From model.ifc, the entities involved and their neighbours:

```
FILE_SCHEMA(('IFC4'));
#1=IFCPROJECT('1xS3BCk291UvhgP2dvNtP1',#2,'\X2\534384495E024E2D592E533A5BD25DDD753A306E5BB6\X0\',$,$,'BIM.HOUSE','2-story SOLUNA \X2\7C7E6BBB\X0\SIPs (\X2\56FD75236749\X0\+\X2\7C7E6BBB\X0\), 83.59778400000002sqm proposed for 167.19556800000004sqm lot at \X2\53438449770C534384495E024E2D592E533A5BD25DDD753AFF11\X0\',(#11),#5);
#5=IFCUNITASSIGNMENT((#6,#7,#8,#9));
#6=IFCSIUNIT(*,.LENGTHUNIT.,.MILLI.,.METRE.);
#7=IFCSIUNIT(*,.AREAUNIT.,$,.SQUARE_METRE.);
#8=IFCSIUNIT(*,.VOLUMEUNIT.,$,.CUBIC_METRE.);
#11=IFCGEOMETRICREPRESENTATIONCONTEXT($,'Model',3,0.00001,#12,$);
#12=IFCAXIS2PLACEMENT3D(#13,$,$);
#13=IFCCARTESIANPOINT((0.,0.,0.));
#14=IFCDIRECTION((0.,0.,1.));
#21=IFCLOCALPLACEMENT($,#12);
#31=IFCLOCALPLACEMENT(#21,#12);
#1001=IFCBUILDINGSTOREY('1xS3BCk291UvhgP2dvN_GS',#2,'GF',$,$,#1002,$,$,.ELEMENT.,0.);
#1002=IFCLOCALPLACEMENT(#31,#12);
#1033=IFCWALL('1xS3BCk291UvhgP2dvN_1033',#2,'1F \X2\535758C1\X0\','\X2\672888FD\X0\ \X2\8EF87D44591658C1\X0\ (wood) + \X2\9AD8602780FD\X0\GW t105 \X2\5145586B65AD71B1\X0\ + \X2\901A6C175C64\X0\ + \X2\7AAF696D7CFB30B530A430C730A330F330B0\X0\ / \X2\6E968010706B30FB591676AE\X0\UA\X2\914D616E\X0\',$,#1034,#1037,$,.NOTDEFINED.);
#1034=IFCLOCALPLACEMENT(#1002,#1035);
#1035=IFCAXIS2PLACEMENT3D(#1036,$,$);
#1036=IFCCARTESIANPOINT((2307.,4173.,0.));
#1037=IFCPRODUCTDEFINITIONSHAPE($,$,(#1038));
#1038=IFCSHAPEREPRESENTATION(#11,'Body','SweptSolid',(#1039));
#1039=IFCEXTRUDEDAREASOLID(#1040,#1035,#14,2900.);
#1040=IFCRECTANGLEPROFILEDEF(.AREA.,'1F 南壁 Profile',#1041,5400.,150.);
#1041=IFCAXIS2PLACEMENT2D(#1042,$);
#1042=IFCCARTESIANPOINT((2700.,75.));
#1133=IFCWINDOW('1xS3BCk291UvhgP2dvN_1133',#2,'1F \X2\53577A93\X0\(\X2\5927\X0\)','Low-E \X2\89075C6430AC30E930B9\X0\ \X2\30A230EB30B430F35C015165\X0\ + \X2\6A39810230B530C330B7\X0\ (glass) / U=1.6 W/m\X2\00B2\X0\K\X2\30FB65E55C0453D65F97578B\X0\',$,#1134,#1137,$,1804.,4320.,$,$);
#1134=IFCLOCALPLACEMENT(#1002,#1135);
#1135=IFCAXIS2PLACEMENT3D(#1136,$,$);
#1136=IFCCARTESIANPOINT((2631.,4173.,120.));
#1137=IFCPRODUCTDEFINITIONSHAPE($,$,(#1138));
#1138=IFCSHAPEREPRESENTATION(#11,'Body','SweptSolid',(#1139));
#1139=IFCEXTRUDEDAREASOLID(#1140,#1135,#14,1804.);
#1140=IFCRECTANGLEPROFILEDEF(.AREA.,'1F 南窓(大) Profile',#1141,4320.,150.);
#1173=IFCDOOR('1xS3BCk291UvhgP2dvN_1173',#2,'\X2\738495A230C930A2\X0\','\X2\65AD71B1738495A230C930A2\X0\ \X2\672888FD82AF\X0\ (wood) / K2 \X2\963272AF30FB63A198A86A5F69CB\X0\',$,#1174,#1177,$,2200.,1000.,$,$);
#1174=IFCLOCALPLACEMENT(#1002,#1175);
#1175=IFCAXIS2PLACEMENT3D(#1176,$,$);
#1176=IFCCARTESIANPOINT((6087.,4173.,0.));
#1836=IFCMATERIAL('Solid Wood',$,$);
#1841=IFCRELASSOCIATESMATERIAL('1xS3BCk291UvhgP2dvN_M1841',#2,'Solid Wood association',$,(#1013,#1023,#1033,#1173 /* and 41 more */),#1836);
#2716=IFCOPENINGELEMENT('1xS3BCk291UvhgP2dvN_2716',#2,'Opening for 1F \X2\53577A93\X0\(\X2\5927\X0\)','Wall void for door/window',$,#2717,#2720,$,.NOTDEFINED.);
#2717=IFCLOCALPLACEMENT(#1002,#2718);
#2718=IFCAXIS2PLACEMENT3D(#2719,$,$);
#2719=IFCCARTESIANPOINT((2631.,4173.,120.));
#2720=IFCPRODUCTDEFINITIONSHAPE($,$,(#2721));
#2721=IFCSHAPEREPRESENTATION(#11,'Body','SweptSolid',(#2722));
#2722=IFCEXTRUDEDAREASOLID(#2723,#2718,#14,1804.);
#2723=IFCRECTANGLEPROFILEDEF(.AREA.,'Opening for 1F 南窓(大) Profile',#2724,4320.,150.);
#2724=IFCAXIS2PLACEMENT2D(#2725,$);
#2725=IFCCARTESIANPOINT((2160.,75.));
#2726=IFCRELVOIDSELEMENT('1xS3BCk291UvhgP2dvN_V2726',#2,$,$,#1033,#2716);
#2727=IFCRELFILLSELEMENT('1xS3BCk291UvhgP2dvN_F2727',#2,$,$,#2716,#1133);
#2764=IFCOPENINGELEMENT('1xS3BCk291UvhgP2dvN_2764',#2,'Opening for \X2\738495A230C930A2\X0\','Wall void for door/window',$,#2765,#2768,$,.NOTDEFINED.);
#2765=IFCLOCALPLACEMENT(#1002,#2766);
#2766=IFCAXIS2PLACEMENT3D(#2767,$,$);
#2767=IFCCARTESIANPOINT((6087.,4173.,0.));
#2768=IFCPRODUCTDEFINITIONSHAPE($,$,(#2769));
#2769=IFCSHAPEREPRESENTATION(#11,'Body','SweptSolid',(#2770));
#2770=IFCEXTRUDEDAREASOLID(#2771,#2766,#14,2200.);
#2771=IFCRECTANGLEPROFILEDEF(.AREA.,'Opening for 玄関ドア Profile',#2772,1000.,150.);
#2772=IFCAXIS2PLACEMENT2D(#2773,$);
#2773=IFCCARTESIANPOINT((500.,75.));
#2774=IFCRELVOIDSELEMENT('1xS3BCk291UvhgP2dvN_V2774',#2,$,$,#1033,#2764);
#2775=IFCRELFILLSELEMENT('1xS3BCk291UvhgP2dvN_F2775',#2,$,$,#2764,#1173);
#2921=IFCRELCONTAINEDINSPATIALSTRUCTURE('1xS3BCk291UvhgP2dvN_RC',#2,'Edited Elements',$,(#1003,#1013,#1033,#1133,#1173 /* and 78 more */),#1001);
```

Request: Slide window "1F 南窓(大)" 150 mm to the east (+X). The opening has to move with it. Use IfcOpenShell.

```python
import ifcopenshell
import ifcopenshell.api.geometry
import ifcopenshell.util.placement

model = ifcopenshell.open("model.ifc")

window = model.by_guid("1xS3BCk291UvhgP2dvN_1133")
opening = window.FillsVoids[0].RelatingOpeningElement
wall = opening.VoidsElements[0].RelatingBuildingElement

wall_matrix = ifcopenshell.util.placement.get_local_placement(wall.ObjectPlacement)
shift = wall_matrix[:3, 0] * 150.0
before = ifcopenshell.util.placement.get_local_placement(window.ObjectPlacement)[:3, 3].copy()

# The window is not placed relative to its opening, so move both.
for product in (opening, window):
    matrix = ifcopenshell.util.placement.get_local_placement(product.ObjectPlacement)
    matrix[:3, 3] += shift
    ifcopenshell.api.geometry.edit_object_placement(model, product=product, matrix=matrix, is_si=False)

after = ifcopenshell.util.placement.get_local_placement(window.ObjectPlacement)[:3, 3]
print("window moved by", (after - before).round(3) + 0.0)

model.write("model_updated.ifc")
```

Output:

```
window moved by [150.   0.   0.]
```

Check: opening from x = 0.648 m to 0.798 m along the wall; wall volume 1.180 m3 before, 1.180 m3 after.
